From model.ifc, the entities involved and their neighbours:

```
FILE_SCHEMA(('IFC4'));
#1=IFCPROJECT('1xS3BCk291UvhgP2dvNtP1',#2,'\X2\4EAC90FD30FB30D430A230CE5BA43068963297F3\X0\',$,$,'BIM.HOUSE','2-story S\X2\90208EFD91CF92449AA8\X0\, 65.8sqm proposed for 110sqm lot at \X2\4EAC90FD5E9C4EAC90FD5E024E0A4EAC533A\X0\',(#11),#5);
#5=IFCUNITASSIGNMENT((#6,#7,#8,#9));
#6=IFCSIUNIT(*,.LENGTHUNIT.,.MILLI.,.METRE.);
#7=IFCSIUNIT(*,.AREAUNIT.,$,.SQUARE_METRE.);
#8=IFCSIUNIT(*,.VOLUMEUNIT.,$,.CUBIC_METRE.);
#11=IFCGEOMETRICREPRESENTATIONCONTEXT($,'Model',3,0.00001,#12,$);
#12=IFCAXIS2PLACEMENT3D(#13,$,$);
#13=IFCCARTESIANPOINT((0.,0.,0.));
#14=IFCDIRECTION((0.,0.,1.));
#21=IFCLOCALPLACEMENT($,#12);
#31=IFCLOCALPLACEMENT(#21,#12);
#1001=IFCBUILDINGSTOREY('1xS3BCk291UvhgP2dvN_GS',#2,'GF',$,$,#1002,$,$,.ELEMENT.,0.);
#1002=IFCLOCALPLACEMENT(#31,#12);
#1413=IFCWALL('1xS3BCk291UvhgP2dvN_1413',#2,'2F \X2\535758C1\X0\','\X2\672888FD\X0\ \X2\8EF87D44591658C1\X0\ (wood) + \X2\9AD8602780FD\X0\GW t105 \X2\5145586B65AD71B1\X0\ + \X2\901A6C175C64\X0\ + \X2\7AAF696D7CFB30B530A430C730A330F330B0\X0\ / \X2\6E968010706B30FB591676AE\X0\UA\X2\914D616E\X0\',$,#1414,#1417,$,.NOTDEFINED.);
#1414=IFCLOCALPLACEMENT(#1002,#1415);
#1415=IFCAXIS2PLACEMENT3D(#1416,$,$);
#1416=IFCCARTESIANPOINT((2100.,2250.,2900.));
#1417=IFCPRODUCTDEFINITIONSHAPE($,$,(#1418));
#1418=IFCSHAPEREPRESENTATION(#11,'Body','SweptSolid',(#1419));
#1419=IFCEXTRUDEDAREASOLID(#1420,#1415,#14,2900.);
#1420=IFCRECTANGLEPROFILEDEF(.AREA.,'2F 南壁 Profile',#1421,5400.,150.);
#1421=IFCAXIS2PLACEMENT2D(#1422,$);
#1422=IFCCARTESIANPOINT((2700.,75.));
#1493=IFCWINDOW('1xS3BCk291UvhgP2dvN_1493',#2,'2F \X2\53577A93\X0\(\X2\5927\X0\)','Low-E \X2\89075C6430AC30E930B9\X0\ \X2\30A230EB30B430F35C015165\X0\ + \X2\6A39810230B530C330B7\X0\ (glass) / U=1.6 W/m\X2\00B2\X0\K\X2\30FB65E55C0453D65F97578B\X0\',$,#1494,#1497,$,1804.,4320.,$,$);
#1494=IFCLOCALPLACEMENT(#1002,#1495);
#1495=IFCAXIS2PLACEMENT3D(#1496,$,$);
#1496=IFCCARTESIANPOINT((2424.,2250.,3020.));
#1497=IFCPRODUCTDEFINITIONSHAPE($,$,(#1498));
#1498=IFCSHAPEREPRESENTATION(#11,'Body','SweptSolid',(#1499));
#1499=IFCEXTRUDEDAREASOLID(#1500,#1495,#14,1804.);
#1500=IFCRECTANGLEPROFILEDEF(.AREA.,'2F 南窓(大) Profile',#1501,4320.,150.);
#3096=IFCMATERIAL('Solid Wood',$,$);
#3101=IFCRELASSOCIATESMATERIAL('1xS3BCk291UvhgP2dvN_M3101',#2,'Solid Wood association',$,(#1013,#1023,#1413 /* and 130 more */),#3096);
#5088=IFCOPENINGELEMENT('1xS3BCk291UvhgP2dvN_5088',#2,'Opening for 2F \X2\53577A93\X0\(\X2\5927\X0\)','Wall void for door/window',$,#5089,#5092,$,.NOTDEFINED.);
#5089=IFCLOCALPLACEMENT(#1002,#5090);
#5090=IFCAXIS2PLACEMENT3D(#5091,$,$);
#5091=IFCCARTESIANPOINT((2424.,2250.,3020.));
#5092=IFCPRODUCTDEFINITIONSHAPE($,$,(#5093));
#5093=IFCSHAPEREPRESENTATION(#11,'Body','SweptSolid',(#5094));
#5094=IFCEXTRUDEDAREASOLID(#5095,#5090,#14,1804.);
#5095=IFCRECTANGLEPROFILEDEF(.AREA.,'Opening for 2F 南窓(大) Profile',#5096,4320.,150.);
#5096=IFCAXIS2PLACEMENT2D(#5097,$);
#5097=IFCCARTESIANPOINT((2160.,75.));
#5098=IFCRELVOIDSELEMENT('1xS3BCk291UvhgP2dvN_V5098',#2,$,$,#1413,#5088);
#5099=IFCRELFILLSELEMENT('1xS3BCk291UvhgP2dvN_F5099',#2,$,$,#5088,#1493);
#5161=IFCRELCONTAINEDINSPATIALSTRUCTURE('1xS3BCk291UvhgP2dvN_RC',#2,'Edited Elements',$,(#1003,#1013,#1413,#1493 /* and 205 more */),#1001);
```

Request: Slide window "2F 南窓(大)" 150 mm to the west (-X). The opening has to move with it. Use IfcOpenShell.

```python
import ifcopenshell
import ifcopenshell.api.geometry
import ifcopenshell.util.placement
import ifcopenshell.util.unit

model = ifcopenshell.open("model.ifc")
unit_scale = ifcopenshell.util.unit.calculate_unit_scale(model)

window = model.by_guid("1xS3BCk291UvhgP2dvN_1493")
opening = window.FillsVoids[0].RelatingOpeningElement
wall = opening.VoidsElements[0].RelatingBuildingElement

wall_matrix = ifcopenshell.util.placement.get_local_placement(wall.ObjectPlacement)
shift = wall_matrix[:3, 0] * -0.15 / unit_scale
before = ifcopenshell.util.placement.get_local_placement(window.ObjectPlacement)[:3, 3].copy()

# The window is not placed relative to its opening, so move both.
for product in (opening, window):
    matrix = ifcopenshell.util.placement.get_local_placement(product.ObjectPlacement)
    matrix[:3, 3] += shift
    ifcopenshell.api.geometry.edit_object_placement(model, product=product, matrix=matrix, is_si=False)

after = ifcopenshell.util.placement.get_local_placement(window.ObjectPlacement)[:3, 3]
print("window moved by", (after - before).round(3) + 0.0)

model.write("model_v2.ifc")
```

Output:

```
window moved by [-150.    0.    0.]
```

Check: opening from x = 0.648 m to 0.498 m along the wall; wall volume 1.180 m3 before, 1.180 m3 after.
